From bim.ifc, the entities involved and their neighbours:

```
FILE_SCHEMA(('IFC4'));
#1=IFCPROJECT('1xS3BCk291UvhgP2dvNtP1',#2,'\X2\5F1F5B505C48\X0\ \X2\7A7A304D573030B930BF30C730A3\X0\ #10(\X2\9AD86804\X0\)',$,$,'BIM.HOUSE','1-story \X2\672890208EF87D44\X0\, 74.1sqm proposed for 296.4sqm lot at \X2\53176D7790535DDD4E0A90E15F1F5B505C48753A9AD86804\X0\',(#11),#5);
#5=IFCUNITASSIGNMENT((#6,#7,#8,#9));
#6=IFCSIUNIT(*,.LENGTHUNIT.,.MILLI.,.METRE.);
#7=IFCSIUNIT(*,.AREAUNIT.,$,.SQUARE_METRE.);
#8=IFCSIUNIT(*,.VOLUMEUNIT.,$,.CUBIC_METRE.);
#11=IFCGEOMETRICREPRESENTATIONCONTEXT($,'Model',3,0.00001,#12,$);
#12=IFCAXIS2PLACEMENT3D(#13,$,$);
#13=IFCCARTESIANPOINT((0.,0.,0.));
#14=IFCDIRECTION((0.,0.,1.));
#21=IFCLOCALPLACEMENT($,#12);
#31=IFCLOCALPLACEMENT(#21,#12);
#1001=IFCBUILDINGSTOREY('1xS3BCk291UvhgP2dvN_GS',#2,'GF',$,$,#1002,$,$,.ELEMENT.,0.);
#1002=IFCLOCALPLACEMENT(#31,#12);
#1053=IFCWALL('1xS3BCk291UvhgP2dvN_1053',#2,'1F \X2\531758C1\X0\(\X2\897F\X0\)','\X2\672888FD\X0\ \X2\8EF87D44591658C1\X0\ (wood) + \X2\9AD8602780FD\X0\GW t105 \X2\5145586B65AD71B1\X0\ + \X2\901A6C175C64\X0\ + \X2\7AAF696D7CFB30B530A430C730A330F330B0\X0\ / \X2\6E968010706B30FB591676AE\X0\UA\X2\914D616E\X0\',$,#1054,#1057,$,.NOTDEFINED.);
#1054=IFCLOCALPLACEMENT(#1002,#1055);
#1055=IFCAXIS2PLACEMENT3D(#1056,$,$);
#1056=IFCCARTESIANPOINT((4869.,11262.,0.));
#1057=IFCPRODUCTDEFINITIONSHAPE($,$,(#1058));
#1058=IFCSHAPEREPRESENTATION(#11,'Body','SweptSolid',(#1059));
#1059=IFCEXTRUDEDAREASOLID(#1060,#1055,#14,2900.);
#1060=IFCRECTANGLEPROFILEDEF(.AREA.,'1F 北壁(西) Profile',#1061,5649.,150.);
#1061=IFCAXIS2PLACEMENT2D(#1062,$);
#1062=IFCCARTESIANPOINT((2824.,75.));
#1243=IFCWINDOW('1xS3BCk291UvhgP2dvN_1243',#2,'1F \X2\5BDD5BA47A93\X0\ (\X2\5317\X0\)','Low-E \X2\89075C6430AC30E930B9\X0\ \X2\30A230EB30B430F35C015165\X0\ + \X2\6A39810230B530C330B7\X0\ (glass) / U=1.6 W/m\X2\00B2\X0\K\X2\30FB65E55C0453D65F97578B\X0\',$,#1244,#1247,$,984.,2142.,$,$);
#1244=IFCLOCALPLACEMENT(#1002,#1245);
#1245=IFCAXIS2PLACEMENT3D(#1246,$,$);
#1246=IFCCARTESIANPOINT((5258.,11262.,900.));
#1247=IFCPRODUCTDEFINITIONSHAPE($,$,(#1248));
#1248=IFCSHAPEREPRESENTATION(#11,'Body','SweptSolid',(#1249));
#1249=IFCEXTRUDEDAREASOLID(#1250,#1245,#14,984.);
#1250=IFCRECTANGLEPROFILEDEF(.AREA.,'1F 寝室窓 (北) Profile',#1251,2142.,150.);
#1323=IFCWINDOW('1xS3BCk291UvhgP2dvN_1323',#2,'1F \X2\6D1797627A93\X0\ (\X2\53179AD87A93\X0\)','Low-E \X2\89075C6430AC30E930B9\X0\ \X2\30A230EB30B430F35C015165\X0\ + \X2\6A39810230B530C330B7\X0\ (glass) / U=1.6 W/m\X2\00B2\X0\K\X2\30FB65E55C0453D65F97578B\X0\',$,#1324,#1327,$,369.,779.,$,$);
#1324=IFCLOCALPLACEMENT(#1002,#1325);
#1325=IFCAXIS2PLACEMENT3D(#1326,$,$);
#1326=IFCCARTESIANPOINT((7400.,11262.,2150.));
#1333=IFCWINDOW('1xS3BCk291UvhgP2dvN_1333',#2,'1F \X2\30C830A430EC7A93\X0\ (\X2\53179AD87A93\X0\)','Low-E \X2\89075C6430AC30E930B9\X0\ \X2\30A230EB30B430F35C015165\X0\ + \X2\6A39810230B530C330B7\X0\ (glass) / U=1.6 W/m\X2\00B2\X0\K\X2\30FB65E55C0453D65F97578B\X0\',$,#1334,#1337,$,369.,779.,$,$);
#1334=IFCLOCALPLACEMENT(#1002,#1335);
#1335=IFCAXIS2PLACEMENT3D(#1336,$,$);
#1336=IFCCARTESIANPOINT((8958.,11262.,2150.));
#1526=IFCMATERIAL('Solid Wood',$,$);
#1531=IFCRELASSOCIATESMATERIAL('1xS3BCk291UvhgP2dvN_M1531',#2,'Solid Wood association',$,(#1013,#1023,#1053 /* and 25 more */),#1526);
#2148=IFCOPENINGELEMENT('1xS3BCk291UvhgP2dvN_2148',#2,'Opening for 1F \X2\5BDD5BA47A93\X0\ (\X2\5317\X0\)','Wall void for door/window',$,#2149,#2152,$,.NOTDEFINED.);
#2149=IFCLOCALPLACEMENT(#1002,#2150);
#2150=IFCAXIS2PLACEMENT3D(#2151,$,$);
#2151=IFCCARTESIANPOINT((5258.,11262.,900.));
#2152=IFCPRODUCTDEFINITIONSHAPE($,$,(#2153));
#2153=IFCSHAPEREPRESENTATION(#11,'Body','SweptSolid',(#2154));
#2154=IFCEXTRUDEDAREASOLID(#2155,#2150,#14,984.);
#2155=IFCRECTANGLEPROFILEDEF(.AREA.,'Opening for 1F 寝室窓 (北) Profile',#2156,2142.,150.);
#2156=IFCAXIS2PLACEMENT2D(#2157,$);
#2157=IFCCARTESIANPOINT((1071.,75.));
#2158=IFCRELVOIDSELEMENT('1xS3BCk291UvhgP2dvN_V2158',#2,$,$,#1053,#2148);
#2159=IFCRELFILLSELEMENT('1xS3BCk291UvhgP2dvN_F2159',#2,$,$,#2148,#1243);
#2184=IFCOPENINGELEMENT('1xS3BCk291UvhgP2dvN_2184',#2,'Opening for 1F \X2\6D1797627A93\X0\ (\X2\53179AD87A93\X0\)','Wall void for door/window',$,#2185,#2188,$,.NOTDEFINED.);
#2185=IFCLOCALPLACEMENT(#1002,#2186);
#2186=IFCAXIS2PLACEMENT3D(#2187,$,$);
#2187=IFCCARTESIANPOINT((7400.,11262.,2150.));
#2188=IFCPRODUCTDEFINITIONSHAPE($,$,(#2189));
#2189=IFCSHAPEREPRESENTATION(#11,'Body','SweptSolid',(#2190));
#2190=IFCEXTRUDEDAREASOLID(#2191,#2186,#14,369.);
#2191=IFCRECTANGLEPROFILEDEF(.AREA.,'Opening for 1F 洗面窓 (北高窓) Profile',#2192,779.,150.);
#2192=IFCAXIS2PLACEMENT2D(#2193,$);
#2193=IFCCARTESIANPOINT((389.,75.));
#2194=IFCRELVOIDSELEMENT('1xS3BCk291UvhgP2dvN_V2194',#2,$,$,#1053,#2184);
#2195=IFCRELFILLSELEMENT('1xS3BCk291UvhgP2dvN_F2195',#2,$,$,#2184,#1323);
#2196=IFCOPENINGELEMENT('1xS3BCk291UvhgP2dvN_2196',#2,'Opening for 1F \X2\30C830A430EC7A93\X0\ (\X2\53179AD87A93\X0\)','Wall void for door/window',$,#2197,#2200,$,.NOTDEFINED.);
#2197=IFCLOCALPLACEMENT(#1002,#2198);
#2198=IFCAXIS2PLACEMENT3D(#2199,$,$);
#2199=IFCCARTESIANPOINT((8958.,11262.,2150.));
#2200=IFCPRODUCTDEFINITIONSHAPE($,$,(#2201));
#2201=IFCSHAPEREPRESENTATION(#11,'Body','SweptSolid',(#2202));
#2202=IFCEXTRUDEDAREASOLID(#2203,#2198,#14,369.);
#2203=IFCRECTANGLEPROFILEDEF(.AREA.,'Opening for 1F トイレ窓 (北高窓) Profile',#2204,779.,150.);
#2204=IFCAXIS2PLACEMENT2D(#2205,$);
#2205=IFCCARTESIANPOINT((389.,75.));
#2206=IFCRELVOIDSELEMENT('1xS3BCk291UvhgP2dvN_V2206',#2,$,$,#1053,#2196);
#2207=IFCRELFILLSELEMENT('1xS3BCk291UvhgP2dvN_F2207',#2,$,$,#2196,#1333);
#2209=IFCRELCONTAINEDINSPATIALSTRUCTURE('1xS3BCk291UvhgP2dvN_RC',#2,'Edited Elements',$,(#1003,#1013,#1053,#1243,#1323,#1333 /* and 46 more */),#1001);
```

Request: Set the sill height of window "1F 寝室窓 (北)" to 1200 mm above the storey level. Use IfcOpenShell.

```python
import numpy as np
import ifcopenshell
import ifcopenshell.api.geometry
import ifcopenshell.geom
import ifcopenshell.util.element
import ifcopenshell.util.placement
import ifcopenshell.util.shape
import ifcopenshell.util.unit

model = ifcopenshell.open("bim.ifc")
unit_scale = ifcopenshell.util.unit.calculate_unit_scale(model)

window = model.by_guid("1xS3BCk291UvhgP2dvN_1243")
opening = window.FillsVoids[0].RelatingOpeningElement
storey = ifcopenshell.util.element.get_container(window, ifc_class="IfcBuildingStorey")
level = ifcopenshell.util.placement.get_local_placement(storey.ObjectPlacement)[2, 3]

# The opening's origin need not be at the sill, so measure its lowest point.
shape = ifcopenshell.geom.create_shape(ifcopenshell.geom.settings(), opening)
bottom = ifcopenshell.util.shape.get_shape_bottom_elevation(shape, shape.geometry) / unit_scale
dz = level + 1.2 / unit_scale - bottom

shift = np.array([0.0, 0.0, dz])
# The window is not placed relative to its opening, so move both.
for product in (opening, window):
    matrix = ifcopenshell.util.placement.get_local_placement(product.ObjectPlacement)
    matrix[:3, 3] += shift
    ifcopenshell.api.geometry.edit_object_placement(model, product=product, matrix=matrix, is_si=False)

print(f"moved by {dz * unit_scale:+.3f} m")

model.write("bim_edited.ifc")
```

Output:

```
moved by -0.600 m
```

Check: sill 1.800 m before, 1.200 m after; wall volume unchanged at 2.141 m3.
